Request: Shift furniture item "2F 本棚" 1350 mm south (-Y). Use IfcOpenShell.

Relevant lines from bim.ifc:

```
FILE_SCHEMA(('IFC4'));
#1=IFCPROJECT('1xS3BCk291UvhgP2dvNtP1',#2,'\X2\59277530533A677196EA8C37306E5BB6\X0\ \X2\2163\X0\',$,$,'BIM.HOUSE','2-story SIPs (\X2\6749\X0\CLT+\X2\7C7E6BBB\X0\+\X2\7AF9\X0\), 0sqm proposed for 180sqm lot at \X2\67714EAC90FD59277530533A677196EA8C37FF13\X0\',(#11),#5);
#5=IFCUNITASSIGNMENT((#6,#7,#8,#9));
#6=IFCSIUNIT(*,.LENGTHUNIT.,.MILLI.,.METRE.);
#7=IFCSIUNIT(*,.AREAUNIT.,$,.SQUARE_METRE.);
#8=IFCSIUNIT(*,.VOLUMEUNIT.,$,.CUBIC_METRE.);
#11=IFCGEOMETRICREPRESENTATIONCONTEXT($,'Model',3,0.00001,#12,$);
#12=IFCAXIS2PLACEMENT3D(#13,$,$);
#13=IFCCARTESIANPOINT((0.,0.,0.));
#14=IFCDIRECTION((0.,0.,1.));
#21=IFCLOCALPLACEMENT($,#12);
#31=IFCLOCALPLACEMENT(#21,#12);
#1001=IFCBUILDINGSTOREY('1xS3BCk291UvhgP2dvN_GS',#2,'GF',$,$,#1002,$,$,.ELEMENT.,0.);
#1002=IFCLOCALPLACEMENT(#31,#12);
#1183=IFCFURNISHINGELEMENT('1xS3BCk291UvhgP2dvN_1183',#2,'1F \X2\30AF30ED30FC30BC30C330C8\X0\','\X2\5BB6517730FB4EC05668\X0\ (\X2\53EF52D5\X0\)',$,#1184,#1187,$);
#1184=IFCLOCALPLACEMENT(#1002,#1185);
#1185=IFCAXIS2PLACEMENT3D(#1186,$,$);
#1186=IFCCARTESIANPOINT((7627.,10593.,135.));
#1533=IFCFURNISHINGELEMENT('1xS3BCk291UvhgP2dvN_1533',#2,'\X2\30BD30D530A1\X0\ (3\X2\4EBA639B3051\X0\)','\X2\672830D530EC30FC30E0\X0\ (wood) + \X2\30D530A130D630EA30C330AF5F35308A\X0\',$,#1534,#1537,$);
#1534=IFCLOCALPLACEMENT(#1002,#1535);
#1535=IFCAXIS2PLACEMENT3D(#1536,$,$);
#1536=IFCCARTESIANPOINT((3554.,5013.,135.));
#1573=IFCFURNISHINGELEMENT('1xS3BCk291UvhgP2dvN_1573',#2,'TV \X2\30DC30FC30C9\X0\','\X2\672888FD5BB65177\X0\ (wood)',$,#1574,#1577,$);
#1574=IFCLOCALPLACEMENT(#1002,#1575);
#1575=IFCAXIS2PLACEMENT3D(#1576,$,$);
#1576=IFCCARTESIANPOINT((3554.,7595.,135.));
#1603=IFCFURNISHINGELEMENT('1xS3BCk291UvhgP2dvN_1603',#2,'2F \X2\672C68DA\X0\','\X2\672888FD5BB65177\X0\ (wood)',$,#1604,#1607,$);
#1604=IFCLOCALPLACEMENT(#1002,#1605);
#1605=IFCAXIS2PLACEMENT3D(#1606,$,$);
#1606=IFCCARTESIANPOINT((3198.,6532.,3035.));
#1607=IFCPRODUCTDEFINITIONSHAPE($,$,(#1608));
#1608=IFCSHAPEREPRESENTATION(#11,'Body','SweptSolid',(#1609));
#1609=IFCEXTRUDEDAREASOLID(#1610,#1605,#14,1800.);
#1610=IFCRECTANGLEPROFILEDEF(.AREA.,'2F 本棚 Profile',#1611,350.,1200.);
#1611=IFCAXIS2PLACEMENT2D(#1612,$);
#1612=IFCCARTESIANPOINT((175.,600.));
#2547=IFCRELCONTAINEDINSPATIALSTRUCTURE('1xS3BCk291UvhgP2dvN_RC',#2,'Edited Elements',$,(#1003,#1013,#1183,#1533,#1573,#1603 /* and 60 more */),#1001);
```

```python
import ifcopenshell
import ifcopenshell.api.geometry
import ifcopenshell.util.placement
import ifcopenshell.util.unit

model = ifcopenshell.open("bim.ifc")
unit_scale = ifcopenshell.util.unit.calculate_unit_scale(model)

item = model.by_guid("1xS3BCk291UvhgP2dvN_1603")
matrix = ifcopenshell.util.placement.get_local_placement(item.ObjectPlacement)
matrix[1, 3] -= 1.35 / unit_scale
ifcopenshell.api.geometry.edit_object_placement(model, product=item, matrix=matrix, is_si=False)

print(ifcopenshell.util.placement.get_local_placement(item.ObjectPlacement).round(3) + 0.0)

model.write("bim-out.ifc")
```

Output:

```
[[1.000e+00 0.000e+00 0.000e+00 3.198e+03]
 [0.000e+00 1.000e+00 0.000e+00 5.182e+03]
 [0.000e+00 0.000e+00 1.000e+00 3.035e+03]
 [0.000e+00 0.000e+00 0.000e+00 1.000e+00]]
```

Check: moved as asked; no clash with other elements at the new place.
